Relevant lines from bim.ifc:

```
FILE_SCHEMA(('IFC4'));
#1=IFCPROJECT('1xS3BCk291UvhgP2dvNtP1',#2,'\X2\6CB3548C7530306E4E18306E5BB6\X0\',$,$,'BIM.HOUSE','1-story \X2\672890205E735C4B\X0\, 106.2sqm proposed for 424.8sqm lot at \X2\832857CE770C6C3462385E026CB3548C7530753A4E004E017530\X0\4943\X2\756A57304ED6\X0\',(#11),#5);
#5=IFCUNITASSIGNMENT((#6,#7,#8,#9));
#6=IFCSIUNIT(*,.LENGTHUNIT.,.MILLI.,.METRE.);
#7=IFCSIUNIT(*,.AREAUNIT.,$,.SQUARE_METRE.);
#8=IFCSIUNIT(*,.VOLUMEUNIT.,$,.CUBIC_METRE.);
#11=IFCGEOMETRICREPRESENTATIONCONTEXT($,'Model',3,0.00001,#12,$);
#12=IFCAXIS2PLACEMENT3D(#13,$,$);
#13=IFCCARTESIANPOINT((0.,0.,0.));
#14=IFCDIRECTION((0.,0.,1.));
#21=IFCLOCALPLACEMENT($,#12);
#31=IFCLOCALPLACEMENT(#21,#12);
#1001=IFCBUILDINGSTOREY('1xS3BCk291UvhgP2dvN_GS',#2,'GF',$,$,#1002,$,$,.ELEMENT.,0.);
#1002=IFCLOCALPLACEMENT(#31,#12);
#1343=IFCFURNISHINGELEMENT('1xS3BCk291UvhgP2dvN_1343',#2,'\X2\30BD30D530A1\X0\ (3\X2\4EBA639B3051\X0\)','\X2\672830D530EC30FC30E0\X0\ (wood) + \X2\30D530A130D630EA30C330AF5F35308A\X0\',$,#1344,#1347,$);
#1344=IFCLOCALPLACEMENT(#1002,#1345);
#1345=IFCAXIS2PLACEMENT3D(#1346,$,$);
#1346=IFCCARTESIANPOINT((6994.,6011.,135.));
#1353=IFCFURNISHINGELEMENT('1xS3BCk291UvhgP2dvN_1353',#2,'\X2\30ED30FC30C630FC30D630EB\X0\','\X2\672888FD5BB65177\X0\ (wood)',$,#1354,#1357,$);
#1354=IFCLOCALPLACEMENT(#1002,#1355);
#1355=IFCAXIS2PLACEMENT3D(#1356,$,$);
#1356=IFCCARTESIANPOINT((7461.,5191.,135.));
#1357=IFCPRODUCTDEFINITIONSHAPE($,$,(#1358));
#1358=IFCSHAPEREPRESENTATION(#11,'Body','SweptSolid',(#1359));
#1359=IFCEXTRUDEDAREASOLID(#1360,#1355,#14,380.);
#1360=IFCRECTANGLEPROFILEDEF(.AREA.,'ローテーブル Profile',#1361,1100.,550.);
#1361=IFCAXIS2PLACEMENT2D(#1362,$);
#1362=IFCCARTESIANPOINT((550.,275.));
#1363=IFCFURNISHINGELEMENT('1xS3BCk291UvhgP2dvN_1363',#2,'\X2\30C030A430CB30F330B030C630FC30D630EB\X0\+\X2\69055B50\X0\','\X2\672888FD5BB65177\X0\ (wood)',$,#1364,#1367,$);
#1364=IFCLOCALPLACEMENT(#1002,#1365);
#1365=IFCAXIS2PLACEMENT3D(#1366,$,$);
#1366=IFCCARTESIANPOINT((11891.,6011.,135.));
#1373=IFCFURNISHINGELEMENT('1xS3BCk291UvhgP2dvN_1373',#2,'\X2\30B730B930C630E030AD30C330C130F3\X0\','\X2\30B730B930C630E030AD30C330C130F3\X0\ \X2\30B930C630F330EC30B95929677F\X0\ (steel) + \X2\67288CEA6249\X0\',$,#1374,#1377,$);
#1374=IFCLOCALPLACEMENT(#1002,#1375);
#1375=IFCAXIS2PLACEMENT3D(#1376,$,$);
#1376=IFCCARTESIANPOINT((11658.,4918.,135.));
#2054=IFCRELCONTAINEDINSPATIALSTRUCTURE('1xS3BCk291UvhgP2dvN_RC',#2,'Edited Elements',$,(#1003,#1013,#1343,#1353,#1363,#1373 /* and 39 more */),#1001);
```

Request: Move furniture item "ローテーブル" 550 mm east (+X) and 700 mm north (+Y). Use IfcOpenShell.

```python
import ifcopenshell
import ifcopenshell.api.geometry
import ifcopenshell.util.placement
import ifcopenshell.util.unit

model = ifcopenshell.open("bim.ifc")
unit_scale = ifcopenshell.util.unit.calculate_unit_scale(model)

item = model.by_guid("1xS3BCk291UvhgP2dvN_1353")
matrix = ifcopenshell.util.placement.get_local_placement(item.ObjectPlacement)
matrix[0, 3] += 0.55 / unit_scale
matrix[1, 3] += 0.7 / unit_scale
ifcopenshell.api.geometry.edit_object_placement(model, product=item, matrix=matrix, is_si=False)

print(ifcopenshell.util.placement.get_local_placement(item.ObjectPlacement).round(3) + 0.0)

model.write("bim_rev.ifc")
```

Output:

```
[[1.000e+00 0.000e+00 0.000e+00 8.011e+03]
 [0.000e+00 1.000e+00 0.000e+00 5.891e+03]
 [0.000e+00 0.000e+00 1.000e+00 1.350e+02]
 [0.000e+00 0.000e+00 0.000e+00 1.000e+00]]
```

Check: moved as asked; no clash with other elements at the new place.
